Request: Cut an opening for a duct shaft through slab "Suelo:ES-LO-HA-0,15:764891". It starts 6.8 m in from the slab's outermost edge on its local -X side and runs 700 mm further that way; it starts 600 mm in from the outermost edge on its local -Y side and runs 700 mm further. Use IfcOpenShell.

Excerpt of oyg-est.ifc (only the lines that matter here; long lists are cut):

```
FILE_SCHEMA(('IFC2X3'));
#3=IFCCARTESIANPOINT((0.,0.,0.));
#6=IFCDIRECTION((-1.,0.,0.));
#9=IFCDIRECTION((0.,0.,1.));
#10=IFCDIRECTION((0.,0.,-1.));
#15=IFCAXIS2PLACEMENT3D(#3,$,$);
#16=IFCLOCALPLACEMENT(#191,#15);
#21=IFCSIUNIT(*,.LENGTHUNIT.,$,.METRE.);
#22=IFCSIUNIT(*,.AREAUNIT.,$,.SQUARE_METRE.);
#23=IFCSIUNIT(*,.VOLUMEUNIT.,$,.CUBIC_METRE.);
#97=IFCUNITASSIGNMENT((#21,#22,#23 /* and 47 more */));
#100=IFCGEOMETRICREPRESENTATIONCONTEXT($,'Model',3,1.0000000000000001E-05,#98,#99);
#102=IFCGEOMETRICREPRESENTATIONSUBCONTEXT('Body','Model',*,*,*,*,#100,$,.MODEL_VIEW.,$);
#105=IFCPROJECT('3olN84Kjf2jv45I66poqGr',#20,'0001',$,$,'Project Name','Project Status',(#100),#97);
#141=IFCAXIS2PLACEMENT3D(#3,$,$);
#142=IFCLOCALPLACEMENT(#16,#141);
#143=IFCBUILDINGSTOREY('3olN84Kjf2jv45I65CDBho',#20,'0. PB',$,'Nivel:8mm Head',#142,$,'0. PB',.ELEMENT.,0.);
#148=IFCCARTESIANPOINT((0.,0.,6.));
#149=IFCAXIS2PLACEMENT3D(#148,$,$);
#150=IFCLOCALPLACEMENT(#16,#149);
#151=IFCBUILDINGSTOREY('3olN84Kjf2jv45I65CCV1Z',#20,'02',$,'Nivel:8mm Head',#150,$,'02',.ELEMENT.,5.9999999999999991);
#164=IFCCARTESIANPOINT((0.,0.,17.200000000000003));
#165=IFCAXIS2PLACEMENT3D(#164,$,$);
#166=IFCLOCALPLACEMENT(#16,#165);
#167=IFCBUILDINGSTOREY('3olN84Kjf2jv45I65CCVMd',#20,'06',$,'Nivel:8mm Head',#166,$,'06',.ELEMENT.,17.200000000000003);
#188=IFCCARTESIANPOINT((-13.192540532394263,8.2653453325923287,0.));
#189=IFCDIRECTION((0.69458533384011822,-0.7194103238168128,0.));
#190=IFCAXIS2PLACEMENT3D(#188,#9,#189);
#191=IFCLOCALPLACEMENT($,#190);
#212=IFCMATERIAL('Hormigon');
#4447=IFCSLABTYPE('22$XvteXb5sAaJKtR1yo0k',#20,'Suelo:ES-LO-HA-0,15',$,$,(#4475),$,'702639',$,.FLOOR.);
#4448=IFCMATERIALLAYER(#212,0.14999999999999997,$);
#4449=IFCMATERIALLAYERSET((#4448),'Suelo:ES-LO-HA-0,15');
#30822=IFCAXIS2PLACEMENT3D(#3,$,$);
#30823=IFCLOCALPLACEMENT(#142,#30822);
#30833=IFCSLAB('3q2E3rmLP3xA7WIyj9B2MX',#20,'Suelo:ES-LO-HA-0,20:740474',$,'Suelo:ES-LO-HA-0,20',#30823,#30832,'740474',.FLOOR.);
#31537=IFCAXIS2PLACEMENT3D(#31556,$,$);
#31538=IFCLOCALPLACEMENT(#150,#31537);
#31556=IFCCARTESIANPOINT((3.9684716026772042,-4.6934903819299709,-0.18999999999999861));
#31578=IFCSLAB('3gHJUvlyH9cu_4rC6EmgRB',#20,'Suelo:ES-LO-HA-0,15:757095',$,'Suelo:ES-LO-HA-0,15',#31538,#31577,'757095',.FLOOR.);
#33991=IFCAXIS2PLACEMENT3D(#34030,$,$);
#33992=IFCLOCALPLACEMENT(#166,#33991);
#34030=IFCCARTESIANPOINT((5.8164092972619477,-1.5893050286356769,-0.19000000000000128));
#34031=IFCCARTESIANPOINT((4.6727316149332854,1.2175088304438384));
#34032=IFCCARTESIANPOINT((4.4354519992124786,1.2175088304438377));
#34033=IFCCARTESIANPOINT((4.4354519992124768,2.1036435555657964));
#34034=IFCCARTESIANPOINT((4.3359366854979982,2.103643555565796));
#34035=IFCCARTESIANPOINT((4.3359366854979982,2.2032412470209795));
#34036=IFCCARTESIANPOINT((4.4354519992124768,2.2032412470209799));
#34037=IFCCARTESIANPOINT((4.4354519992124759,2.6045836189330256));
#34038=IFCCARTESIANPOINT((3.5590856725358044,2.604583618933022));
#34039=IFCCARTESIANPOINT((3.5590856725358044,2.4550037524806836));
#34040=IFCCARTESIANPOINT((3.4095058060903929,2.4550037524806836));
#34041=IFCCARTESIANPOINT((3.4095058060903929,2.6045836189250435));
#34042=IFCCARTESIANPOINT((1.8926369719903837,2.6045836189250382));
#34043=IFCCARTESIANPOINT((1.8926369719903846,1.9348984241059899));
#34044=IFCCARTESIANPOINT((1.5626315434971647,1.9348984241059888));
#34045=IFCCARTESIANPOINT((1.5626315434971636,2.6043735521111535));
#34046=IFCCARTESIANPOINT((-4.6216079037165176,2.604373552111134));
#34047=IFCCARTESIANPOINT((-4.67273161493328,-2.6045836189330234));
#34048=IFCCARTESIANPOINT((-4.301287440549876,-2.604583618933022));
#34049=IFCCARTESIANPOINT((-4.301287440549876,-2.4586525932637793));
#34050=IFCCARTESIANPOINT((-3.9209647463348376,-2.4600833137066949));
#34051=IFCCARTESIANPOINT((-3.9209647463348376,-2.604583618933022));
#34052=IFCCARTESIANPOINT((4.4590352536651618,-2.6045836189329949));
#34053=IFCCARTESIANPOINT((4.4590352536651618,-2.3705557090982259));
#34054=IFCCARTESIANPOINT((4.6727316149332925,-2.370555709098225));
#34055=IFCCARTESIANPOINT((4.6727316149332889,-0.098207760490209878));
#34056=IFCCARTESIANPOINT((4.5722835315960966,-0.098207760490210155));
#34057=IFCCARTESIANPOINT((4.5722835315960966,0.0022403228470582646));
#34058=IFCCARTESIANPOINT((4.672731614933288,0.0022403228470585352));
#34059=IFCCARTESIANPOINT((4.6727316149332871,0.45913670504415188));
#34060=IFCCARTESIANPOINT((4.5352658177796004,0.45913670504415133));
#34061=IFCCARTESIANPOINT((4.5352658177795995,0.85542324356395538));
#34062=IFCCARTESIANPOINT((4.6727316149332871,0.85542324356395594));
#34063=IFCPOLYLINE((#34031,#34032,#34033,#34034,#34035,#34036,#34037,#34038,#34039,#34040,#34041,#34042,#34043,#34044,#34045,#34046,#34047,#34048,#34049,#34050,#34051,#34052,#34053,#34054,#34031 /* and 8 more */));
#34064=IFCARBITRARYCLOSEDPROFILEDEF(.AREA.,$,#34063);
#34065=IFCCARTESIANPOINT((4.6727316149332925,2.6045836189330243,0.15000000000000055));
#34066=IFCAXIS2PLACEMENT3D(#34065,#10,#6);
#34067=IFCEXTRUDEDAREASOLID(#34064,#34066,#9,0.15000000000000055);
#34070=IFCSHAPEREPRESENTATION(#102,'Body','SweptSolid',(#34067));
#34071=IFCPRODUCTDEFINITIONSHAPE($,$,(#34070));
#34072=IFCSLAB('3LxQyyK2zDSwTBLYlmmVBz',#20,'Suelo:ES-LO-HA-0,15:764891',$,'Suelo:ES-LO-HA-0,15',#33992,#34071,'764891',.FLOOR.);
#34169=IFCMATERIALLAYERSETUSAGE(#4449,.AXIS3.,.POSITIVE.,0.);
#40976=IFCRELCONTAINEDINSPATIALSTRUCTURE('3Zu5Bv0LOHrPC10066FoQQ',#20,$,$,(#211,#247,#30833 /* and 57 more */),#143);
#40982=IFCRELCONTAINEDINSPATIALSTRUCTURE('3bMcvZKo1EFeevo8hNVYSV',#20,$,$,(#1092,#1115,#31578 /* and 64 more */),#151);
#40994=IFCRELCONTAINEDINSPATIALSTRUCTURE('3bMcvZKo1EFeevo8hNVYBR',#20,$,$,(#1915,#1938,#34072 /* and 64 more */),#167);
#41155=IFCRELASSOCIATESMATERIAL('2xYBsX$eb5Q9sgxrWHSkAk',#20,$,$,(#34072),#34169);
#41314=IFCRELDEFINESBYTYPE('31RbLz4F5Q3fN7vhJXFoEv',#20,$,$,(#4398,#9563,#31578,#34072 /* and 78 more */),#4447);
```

```python
import numpy as np
import ifcopenshell
import ifcopenshell.api.feature
import ifcopenshell.api.geometry
import ifcopenshell.api.root
import ifcopenshell.geom
import ifcopenshell.util.placement
import ifcopenshell.util.representation
import ifcopenshell.util.shape
import ifcopenshell.util.unit

model = ifcopenshell.open("oyg-est.ifc")
unit_scale = ifcopenshell.util.unit.calculate_unit_scale(model)
settings = ifcopenshell.geom.settings()


def volume(element):
    """Net volume in cubic metres, openings subtracted."""
    shape = ifcopenshell.geom.create_shape(settings, element)
    return ifcopenshell.util.shape.get_volume(shape.geometry)


slab = model.by_id(34072)
before = volume(slab)

# Extent in the slab's own axes, in metres. The edges named are its -X and -Y sides.
slab_shape = ifcopenshell.geom.create_shape(settings, slab)
vertices = ifcopenshell.util.shape.get_vertices(slab_shape.geometry)
x_min, y_min, bottom = vertices.min(axis=0)
top = vertices[:, 2].max()

opening = ifcopenshell.api.root.create_entity(model, ifc_class="IfcOpeningElement", name="Duct shaft opening")
context = ifcopenshell.util.representation.get_context(model, "Model", "Body", "MODEL_VIEW")
width, depth = 0.7, 0.7
outline = [(0.0, 0.0), (width, 0.0), (width, depth), (0.0, depth), (0.0, 0.0)]
# Overshoot both faces by 50 mm so the cut is clean.
shape = ifcopenshell.api.geometry.add_slab_representation(
    model, context=context, depth=top - bottom + 0.1, polyline=outline
)
ifcopenshell.api.geometry.assign_representation(model, product=opening, representation=shape)

matrix = ifcopenshell.util.placement.get_local_placement(slab.ObjectPlacement)
matrix[:, 3] = matrix @ np.append(np.array([x_min + 6.8, y_min + 0.6, bottom - 0.05]) / unit_scale, 1.0)
ifcopenshell.api.geometry.edit_object_placement(model, product=opening, matrix=matrix, is_si=False)
ifcopenshell.api.feature.add_feature(model, feature=opening, element=slab)

after = volume(slab)

print(f"slab volume {before:.3f} -> {after:.3f} m3")

model.write("oyg-est-out.ifc")
```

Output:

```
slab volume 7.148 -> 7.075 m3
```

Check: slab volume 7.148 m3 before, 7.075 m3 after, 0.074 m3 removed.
